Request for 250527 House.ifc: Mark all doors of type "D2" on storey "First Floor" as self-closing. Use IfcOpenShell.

First a look at what the model holds.

```python
import ifcopenshell
import ifcopenshell.util.element

model = ifcopenshell.open("250527 House.ifc")
print(model.schema)
storey = next(s for s in model.by_type("IfcBuildingStorey") if s.Name == "First Floor")
doors = [e for e in ifcopenshell.util.element.get_decomposition(storey) if e.is_a("IfcDoor")]
seen = {}
for e in doors:
    element_type = ifcopenshell.util.element.get_type(e)
    key = (element_type.Name if element_type != e and element_type else None, ifcopenshell.util.element.get_pset(e, "Pset_DoorCommon", "SelfClosing"))
    seen[key] = seen.get(key, 0) + 1
for (name, value), count in sorted(seen.items(), key=str):
    print(count, "x", name, "|", value)
```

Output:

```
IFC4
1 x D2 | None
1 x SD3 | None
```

```python
import ifcopenshell
import ifcopenshell.api.pset
import ifcopenshell.util.element

model = ifcopenshell.open("250527 House.ifc")

storey = next(s for s in model.by_type("IfcBuildingStorey") if s.Name == "First Floor")
doors = [e for e in ifcopenshell.util.element.get_decomposition(storey) if e.is_a("IfcDoor")]

count = 0
for e in doors:
    element_type = ifcopenshell.util.element.get_type(e)
    if element_type in (None, e) or element_type.Name != "D2":
        continue
    # add_pset returns the element's existing set when there is one.
    pset = ifcopenshell.api.pset.add_pset(model, product=e, name="Pset_DoorCommon")
    ifcopenshell.api.pset.edit_pset(model, pset=pset, properties={"SelfClosing": True})
    count += 1

print(count, "doors updated")

model.write("250527 House_updated.ifc")
```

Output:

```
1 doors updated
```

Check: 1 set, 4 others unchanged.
